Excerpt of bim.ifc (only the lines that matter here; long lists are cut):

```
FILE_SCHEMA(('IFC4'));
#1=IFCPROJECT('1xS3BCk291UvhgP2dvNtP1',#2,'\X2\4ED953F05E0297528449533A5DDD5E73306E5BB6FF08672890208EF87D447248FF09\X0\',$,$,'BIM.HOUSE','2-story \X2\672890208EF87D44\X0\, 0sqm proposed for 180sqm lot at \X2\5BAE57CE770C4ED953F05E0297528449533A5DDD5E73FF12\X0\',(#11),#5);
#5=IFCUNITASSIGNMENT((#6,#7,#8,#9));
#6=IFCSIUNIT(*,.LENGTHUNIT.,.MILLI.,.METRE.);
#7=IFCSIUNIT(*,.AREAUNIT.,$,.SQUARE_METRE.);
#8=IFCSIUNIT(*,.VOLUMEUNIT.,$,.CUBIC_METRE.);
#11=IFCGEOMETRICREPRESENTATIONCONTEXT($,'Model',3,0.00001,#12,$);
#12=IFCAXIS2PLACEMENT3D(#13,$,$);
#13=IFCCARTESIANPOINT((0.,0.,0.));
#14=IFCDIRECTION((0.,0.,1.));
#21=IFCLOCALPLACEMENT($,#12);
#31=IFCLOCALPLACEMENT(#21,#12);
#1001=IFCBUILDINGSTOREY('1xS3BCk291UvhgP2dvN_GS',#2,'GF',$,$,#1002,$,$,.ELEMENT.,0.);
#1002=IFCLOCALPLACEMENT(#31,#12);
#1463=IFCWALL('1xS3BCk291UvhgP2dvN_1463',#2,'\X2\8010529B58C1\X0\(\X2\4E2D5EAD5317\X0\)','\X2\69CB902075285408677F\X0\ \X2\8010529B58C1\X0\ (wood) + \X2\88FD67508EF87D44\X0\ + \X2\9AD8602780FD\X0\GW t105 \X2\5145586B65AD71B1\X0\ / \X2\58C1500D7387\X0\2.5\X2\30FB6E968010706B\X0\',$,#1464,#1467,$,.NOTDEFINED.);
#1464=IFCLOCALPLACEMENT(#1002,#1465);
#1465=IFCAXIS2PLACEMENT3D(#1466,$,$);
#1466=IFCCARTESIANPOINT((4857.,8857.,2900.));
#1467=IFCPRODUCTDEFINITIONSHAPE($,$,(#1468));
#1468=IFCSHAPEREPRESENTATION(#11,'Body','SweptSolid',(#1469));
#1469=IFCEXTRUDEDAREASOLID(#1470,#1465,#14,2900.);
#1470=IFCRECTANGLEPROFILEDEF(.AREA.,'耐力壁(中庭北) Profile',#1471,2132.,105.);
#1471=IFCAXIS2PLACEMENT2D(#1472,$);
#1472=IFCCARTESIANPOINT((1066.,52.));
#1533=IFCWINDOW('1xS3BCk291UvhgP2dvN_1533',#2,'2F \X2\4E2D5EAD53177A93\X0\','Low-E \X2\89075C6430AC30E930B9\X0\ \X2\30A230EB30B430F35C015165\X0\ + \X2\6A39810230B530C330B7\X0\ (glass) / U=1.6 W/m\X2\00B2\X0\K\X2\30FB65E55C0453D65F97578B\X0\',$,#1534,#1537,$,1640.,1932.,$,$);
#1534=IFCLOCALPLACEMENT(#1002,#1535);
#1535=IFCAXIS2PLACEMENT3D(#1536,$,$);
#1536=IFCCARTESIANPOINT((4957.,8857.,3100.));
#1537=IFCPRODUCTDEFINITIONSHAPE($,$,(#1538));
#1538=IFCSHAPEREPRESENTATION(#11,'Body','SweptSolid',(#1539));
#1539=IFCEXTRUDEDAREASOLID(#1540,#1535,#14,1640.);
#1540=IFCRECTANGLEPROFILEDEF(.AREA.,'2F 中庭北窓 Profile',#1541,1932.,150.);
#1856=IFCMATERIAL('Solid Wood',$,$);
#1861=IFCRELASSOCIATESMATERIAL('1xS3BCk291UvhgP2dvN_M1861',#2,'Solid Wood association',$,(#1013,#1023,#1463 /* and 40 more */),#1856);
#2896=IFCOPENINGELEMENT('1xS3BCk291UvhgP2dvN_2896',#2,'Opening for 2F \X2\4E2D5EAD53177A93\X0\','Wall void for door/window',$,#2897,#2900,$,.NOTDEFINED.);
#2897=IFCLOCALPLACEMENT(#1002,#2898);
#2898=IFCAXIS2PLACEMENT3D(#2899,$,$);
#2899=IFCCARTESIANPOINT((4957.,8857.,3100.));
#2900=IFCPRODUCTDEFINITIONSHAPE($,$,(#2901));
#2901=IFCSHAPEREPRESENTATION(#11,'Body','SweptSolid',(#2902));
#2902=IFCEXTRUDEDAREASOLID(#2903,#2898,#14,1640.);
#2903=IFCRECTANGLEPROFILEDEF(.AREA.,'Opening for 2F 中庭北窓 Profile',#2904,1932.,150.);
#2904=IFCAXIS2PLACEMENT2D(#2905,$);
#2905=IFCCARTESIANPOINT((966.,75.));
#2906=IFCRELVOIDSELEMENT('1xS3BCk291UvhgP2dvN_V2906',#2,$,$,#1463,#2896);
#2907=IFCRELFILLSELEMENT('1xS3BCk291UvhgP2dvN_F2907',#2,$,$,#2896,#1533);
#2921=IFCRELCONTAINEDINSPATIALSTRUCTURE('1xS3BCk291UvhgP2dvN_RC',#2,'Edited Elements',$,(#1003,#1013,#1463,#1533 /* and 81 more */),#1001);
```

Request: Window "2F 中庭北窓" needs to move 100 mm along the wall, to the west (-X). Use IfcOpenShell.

```python
import ifcopenshell
import ifcopenshell.api.geometry
import ifcopenshell.util.placement
import ifcopenshell.util.unit

model = ifcopenshell.open("bim.ifc")
unit_scale = ifcopenshell.util.unit.calculate_unit_scale(model)

window = model.by_guid("1xS3BCk291UvhgP2dvN_1533")
opening = window.FillsVoids[0].RelatingOpeningElement
wall = opening.VoidsElements[0].RelatingBuildingElement

wall_matrix = ifcopenshell.util.placement.get_local_placement(wall.ObjectPlacement)
shift = wall_matrix[:3, 0] * -0.1 / unit_scale
before = ifcopenshell.util.placement.get_local_placement(window.ObjectPlacement)[:3, 3].copy()

# The window is not placed relative to its opening, so move both.
for product in (opening, window):
    matrix = ifcopenshell.util.placement.get_local_placement(product.ObjectPlacement)
    matrix[:3, 3] += shift
    ifcopenshell.api.geometry.edit_object_placement(model, product=product, matrix=matrix, is_si=False)

after = ifcopenshell.util.placement.get_local_placement(window.ObjectPlacement)[:3, 3]
print("window moved by", (after - before).round(3) + 0.0)

model.write("bim_updated.ifc")
```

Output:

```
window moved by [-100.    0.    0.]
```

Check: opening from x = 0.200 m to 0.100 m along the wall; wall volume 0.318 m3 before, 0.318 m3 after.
